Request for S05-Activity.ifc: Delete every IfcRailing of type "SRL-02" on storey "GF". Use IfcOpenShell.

First a look at what the model holds.

```python
import ifcopenshell
import ifcopenshell.util.element

model = ifcopenshell.open("S05-Activity.ifc")
print(model.schema)
storey = next(s for s in model.by_type("IfcBuildingStorey") if s.Name == "GF")
railings = [e for e in ifcopenshell.util.element.get_decomposition(storey) if e.is_a("IfcRailing")]
seen = {}
for e in railings:
    element_type = ifcopenshell.util.element.get_type(e)
    name = element_type.Name if element_type not in (None, e) else None
    seen[name] = seen.get(name, 0) + 1
for name, count in sorted(seen.items(), key=str):
    print(count, "x", name)
```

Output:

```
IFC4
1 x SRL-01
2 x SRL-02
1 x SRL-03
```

```python
import ifcopenshell
import ifcopenshell.api.root
import ifcopenshell.util.element

model = ifcopenshell.open("S05-Activity.ifc")

storey = next(s for s in model.by_type("IfcBuildingStorey") if s.Name == "GF")
railings = [e for e in ifcopenshell.util.element.get_decomposition(storey) if e.is_a("IfcRailing")]
targets = [e for e in railings if (t := ifcopenshell.util.element.get_type(e)) not in (None, e) and t.Name == "SRL-02"]

for e in targets:
    ifcopenshell.api.root.remove_product(model, product=e)
print(len(targets), "removed")

model.write("S05-Activity_edited.ifc")
```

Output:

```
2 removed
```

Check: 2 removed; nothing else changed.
